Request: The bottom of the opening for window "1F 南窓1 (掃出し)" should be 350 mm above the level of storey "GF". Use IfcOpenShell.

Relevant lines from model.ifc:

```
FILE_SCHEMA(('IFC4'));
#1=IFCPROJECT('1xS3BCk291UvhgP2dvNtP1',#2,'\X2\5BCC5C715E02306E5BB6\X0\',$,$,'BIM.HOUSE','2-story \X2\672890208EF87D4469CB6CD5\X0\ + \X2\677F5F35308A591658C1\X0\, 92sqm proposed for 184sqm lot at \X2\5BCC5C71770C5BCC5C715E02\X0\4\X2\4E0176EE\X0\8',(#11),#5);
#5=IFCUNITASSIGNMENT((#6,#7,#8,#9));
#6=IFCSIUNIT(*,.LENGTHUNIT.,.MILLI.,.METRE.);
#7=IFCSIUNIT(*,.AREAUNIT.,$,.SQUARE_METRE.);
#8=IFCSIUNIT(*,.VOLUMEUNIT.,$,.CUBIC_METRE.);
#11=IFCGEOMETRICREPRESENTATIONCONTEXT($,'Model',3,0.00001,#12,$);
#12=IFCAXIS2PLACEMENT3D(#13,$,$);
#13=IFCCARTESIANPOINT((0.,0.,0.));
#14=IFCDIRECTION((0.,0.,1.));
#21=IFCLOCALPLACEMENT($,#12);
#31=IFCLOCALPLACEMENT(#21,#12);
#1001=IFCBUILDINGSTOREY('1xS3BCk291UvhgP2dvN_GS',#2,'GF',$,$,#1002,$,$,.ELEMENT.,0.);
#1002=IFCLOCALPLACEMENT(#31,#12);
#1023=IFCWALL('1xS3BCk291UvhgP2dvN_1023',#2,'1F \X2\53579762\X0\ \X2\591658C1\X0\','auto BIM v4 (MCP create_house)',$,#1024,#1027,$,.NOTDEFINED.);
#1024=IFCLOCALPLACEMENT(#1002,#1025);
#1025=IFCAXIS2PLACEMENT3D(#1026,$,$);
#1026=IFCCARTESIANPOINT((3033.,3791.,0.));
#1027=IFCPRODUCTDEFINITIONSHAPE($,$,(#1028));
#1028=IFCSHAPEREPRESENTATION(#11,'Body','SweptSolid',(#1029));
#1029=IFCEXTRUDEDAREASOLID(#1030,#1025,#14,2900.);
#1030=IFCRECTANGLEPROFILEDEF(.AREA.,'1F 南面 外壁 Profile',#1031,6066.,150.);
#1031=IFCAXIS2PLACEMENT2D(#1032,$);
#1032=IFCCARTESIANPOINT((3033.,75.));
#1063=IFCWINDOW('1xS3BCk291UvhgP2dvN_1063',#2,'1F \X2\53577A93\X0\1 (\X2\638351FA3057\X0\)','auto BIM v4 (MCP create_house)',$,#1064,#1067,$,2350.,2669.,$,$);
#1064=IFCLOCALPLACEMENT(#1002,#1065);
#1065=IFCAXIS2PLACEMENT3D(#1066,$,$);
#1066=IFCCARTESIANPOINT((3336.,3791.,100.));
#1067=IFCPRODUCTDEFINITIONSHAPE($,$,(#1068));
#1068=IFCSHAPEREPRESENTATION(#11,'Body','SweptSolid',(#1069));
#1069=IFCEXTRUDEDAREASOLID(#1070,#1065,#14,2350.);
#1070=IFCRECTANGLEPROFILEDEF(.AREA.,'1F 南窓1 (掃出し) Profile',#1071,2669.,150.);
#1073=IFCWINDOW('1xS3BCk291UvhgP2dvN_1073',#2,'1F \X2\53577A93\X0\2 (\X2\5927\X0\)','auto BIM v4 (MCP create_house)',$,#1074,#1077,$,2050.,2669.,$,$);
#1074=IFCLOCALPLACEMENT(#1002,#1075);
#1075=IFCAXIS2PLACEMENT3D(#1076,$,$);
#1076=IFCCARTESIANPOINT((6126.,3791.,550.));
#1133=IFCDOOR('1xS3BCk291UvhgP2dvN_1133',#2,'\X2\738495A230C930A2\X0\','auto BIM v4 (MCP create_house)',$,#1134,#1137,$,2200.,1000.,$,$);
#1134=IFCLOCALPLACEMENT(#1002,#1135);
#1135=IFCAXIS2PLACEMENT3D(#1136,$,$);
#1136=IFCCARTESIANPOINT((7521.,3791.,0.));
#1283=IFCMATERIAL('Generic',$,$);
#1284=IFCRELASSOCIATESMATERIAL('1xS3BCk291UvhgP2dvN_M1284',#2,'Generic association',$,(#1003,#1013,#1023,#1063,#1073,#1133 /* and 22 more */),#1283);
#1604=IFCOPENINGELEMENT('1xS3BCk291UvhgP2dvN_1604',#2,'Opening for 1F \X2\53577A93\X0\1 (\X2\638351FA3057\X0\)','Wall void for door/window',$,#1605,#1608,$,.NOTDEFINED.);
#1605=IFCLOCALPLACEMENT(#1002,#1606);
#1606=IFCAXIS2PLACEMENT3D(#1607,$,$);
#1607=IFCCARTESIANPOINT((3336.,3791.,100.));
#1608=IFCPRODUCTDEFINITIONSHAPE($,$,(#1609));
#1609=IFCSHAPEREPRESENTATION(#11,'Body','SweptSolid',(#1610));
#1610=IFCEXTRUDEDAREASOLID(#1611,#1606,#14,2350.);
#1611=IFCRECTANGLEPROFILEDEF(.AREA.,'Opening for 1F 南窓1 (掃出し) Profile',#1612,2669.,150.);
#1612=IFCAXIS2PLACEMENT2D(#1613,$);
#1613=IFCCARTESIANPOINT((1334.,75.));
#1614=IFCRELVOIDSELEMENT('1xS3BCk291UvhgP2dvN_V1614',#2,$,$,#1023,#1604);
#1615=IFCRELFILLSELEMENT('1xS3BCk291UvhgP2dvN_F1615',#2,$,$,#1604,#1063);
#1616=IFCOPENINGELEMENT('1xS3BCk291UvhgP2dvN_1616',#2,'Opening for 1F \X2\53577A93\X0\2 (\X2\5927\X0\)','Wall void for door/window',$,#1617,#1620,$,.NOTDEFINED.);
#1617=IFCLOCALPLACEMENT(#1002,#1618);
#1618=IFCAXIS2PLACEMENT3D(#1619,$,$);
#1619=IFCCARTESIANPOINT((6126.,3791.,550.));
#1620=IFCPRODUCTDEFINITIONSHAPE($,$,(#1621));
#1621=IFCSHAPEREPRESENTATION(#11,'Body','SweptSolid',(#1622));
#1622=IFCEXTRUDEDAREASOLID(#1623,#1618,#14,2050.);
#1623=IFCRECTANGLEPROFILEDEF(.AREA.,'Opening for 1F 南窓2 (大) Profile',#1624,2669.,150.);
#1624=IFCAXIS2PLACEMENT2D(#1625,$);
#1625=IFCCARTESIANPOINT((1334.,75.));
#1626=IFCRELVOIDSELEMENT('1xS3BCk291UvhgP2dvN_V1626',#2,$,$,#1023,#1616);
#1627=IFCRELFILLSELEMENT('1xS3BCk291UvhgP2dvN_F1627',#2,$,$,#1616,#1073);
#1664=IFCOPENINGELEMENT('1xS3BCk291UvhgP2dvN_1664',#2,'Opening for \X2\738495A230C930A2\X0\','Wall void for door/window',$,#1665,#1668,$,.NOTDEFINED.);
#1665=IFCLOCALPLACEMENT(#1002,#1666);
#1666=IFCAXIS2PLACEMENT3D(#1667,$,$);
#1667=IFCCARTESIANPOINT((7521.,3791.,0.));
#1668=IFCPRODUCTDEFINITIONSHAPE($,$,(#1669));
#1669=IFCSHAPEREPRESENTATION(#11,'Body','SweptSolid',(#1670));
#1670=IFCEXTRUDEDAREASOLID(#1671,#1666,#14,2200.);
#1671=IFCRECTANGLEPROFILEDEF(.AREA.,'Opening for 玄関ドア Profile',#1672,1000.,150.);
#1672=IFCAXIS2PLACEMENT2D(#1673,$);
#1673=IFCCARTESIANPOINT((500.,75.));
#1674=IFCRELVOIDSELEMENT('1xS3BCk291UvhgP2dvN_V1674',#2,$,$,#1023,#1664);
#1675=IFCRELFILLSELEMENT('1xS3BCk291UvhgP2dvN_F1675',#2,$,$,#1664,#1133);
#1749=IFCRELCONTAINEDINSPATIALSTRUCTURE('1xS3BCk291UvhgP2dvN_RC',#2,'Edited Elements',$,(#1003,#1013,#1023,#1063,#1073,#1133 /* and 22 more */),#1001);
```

```python
import numpy as np
import ifcopenshell
import ifcopenshell.api.geometry
import ifcopenshell.geom
import ifcopenshell.util.element
import ifcopenshell.util.placement
import ifcopenshell.util.shape
import ifcopenshell.util.unit

model = ifcopenshell.open("model.ifc")
unit_scale = ifcopenshell.util.unit.calculate_unit_scale(model)

window = model.by_guid("1xS3BCk291UvhgP2dvN_1063")
opening = window.FillsVoids[0].RelatingOpeningElement
storey = ifcopenshell.util.element.get_container(window, ifc_class="IfcBuildingStorey")
level = ifcopenshell.util.placement.get_local_placement(storey.ObjectPlacement)[2, 3]

# The opening's origin need not be at the sill, so measure its lowest point.
shape = ifcopenshell.geom.create_shape(ifcopenshell.geom.settings(), opening)
bottom = ifcopenshell.util.shape.get_shape_bottom_elevation(shape, shape.geometry) / unit_scale
dz = level + 0.35 / unit_scale - bottom

shift = np.array([0.0, 0.0, dz])
# The window is not placed relative to its opening, so move both.
for product in (opening, window):
    matrix = ifcopenshell.util.placement.get_local_placement(product.ObjectPlacement)
    matrix[:3, 3] += shift
    ifcopenshell.api.geometry.edit_object_placement(model, product=product, matrix=matrix, is_si=False)

print(f"moved by {dz * unit_scale:+.3f} m")

model.write("model_v2.ifc")
```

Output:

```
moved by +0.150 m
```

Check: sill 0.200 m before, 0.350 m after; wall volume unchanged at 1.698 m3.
